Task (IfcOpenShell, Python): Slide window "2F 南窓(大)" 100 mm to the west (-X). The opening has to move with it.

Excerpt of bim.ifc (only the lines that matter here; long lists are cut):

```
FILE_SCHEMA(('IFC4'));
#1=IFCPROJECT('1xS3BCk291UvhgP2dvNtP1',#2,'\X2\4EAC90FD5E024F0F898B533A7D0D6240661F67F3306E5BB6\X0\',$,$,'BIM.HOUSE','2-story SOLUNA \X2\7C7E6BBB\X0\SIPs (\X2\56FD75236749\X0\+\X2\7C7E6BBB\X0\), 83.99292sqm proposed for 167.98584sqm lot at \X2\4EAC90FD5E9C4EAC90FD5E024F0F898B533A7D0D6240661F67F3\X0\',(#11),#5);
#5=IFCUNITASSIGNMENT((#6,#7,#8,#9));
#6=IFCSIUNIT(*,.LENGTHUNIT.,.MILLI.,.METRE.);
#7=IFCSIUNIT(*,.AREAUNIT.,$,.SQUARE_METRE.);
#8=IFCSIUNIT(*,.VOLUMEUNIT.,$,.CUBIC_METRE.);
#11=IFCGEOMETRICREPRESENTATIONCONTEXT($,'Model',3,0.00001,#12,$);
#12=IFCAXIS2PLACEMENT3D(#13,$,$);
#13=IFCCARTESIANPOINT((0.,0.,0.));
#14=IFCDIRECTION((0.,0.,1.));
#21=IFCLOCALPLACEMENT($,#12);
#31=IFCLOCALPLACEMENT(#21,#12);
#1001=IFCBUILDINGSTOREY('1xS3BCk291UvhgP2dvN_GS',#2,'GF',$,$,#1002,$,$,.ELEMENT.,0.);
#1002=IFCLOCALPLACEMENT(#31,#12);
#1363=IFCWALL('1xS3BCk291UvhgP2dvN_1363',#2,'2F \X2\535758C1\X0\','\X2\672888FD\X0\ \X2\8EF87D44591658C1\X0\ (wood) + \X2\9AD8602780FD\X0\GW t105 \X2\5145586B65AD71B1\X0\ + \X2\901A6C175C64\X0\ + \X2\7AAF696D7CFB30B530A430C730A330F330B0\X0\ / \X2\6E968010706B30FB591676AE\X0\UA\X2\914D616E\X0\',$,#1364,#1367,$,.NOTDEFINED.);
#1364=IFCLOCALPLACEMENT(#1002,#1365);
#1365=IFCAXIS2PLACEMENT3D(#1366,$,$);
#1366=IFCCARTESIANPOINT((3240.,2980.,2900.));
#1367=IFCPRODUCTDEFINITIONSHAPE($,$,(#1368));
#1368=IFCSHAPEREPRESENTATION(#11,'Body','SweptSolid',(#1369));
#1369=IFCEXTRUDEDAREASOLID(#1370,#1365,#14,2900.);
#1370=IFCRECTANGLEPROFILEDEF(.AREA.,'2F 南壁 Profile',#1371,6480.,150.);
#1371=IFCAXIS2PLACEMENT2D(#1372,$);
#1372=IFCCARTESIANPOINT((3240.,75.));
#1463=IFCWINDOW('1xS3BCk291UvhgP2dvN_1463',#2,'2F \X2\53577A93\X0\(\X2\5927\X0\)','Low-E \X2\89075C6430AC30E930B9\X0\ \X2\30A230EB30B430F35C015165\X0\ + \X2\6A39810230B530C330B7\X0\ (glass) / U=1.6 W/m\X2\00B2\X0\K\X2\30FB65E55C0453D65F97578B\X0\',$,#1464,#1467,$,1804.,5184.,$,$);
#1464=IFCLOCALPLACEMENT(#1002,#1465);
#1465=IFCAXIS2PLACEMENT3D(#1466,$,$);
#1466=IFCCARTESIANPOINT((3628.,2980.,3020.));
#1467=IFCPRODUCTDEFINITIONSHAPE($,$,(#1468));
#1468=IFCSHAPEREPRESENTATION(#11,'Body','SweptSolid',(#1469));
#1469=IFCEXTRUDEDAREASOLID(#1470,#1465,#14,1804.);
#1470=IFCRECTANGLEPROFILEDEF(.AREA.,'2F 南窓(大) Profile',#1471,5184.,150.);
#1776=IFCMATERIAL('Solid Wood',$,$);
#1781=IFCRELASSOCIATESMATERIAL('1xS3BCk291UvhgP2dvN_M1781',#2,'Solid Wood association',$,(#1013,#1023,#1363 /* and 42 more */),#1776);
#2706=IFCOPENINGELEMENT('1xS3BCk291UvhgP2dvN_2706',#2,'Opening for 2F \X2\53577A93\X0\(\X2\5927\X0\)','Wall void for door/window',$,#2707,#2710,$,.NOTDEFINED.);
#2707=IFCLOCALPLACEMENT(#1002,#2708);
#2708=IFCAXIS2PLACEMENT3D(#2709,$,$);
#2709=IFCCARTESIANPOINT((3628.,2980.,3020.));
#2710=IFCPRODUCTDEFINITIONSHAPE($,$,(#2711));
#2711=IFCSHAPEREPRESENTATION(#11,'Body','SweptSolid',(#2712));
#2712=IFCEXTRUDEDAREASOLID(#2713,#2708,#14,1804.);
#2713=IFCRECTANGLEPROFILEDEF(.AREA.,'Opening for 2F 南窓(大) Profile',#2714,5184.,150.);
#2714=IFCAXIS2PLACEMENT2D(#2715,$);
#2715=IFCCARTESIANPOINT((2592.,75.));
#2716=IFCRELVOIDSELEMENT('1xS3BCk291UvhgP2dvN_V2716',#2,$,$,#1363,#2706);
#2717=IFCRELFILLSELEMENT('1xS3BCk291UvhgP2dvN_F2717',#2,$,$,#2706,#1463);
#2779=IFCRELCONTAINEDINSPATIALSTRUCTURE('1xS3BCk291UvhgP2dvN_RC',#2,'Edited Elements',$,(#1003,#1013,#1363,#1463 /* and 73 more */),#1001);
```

```python
import ifcopenshell
import ifcopenshell.api.geometry
import ifcopenshell.util.placement
import ifcopenshell.util.unit

model = ifcopenshell.open("bim.ifc")
unit_scale = ifcopenshell.util.unit.calculate_unit_scale(model)

window = model.by_guid("1xS3BCk291UvhgP2dvN_1463")
opening = window.FillsVoids[0].RelatingOpeningElement
wall = opening.VoidsElements[0].RelatingBuildingElement

wall_matrix = ifcopenshell.util.placement.get_local_placement(wall.ObjectPlacement)
shift = wall_matrix[:3, 0] * -0.1 / unit_scale
before = ifcopenshell.util.placement.get_local_placement(window.ObjectPlacement)[:3, 3].copy()

# The window is not placed relative to its opening, so move both.
for product in (opening, window):
    matrix = ifcopenshell.util.placement.get_local_placement(product.ObjectPlacement)
    matrix[:3, 3] += shift
    ifcopenshell.api.geometry.edit_object_placement(model, product=product, matrix=matrix, is_si=False)

after = ifcopenshell.util.placement.get_local_placement(window.ObjectPlacement)[:3, 3]
print("window moved by", (after - before).round(3) + 0.0)

model.write("bim_edited.ifc")
```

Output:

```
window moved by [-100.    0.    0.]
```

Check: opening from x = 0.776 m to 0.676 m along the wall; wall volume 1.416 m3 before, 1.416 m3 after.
